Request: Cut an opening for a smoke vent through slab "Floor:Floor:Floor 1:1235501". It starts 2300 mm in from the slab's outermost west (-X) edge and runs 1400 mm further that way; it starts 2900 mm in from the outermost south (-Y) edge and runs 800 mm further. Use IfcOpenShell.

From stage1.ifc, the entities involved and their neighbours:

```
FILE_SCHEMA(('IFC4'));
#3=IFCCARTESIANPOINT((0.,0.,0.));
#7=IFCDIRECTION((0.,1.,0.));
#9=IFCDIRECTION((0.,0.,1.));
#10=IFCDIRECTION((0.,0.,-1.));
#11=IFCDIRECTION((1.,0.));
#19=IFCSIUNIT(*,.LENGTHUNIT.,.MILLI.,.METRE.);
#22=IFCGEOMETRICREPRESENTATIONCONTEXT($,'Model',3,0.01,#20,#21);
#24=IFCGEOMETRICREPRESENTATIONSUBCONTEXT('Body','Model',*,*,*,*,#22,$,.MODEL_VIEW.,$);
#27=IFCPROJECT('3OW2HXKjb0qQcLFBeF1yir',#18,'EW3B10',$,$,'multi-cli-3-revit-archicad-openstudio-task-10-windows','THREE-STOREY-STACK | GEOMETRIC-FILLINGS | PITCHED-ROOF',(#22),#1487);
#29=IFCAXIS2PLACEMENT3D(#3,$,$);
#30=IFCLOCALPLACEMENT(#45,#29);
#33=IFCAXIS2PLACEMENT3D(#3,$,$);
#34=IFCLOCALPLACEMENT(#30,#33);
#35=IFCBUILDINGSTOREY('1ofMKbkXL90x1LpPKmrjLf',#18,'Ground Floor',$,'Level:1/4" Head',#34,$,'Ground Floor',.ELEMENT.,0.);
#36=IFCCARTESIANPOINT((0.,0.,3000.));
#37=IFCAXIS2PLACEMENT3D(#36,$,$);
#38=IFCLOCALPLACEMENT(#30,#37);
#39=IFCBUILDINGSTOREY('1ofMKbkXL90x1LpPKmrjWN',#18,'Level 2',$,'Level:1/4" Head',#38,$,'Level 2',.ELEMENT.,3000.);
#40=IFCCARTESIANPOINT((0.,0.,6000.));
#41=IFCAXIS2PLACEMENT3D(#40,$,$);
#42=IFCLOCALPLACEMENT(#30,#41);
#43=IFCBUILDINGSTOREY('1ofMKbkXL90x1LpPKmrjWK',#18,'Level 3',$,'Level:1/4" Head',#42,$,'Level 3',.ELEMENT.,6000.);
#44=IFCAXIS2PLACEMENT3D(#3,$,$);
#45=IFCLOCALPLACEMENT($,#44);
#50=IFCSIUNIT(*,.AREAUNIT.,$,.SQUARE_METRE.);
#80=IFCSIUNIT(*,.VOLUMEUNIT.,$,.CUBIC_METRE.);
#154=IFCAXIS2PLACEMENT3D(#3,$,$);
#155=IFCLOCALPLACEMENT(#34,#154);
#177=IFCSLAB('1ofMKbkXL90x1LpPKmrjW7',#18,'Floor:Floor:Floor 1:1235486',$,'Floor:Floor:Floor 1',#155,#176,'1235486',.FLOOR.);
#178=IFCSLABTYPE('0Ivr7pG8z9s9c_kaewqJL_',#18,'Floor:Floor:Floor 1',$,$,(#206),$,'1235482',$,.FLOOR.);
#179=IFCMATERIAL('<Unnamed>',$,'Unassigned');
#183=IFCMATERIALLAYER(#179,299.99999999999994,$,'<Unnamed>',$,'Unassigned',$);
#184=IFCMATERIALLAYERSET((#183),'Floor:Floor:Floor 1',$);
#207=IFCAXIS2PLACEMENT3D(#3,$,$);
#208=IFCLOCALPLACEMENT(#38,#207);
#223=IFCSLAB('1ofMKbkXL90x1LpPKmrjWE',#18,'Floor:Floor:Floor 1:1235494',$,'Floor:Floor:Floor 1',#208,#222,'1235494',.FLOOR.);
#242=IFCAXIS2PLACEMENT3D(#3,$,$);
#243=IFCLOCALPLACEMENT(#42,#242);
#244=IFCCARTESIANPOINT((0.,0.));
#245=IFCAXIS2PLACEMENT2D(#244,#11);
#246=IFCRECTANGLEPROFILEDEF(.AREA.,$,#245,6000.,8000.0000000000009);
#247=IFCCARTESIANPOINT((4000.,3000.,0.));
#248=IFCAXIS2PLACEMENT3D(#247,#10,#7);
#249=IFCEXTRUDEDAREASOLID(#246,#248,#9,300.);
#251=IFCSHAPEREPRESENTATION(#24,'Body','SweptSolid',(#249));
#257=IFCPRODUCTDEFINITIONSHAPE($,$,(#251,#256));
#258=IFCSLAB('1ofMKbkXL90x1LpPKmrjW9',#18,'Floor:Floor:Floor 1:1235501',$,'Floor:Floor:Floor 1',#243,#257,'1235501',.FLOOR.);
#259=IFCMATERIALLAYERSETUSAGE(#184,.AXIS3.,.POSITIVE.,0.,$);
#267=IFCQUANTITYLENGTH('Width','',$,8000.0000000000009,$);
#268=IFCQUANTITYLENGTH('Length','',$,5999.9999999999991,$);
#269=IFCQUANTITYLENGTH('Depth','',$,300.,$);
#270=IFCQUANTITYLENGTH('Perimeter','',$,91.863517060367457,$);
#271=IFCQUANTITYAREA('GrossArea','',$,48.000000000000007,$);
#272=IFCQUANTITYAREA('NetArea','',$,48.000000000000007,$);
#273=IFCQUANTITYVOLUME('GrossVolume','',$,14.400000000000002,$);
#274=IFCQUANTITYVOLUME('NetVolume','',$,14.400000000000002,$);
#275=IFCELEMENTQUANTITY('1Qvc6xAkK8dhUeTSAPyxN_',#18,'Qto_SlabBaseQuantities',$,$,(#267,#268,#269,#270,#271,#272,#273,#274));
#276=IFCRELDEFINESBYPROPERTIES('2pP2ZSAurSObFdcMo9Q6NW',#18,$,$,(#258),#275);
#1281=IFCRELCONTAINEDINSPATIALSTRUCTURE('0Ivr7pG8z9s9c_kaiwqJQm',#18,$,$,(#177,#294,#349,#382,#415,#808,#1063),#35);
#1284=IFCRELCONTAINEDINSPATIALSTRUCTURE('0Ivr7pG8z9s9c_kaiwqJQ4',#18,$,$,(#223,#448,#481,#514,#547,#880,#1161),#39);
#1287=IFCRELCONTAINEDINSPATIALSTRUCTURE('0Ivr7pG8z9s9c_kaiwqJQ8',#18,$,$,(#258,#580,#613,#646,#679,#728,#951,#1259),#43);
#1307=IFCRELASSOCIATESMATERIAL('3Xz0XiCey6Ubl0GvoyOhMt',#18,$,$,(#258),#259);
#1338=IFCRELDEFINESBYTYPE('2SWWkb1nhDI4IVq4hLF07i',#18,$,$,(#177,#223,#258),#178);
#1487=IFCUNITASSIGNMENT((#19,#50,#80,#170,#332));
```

```python
import numpy as np
import ifcopenshell
import ifcopenshell.api.feature
import ifcopenshell.api.geometry
import ifcopenshell.api.pset
import ifcopenshell.api.root
import ifcopenshell.geom
import ifcopenshell.util.element
import ifcopenshell.util.placement
import ifcopenshell.util.representation
import ifcopenshell.util.shape
import ifcopenshell.util.unit

model = ifcopenshell.open("stage1.ifc")
unit_scale = ifcopenshell.util.unit.calculate_unit_scale(model)
area_scale = ifcopenshell.util.unit.calculate_unit_scale(model, "AREAUNIT")
volume_scale = ifcopenshell.util.unit.calculate_unit_scale(model, "VOLUMEUNIT")
settings = ifcopenshell.geom.settings()


def volume(element):
    """Net volume in cubic metres, openings subtracted."""
    shape = ifcopenshell.geom.create_shape(settings, element)
    return ifcopenshell.util.shape.get_volume(shape.geometry)


slab = model.by_guid("1ofMKbkXL90x1LpPKmrjW9")
before = volume(slab)

# Extent in the slab's own axes, in metres. The edges named are its -X and -Y sides.
slab_shape = ifcopenshell.geom.create_shape(settings, slab)
vertices = ifcopenshell.util.shape.get_vertices(slab_shape.geometry)
x_min, y_min, bottom = vertices.min(axis=0)
top = vertices[:, 2].max()

opening = ifcopenshell.api.root.create_entity(model, ifc_class="IfcOpeningElement", name="Smoke vent opening", predefined_type="OPENING")
context = ifcopenshell.util.representation.get_context(model, "Model", "Body", "MODEL_VIEW")
width, depth = 1.4, 0.8
outline = [(0.0, 0.0), (width, 0.0), (width, depth), (0.0, depth), (0.0, 0.0)]
# Overshoot both faces by 50 mm so the cut is clean.
shape = ifcopenshell.api.geometry.add_slab_representation(
    model, context=context, depth=top - bottom + 0.1, polyline=outline
)
ifcopenshell.api.geometry.assign_representation(model, product=opening, representation=shape)

matrix = ifcopenshell.util.placement.get_local_placement(slab.ObjectPlacement)
matrix[:, 3] = matrix @ np.append(np.array([x_min + 2.3, y_min + 2.9, bottom - 0.05]) / unit_scale, 1.0)
ifcopenshell.api.geometry.edit_object_placement(model, product=opening, matrix=matrix, is_si=False)
ifcopenshell.api.feature.add_feature(model, feature=opening, element=slab)

after = volume(slab)

# Update the slab's stored quantities.
qto = model.by_id(ifcopenshell.util.element.get_pset(slab, "Qto_SlabBaseQuantities", should_inherit=False)["id"])
ifcopenshell.api.pset.edit_qto(model, qto=qto, properties={
    "NetArea": after / (top - bottom) / area_scale,
    "NetVolume": after / volume_scale,
})

print(f"slab volume {before:.3f} -> {after:.3f} m3")

model.write("stage1-out.ifc")
```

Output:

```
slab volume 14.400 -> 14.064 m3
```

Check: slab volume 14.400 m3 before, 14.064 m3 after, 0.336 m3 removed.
